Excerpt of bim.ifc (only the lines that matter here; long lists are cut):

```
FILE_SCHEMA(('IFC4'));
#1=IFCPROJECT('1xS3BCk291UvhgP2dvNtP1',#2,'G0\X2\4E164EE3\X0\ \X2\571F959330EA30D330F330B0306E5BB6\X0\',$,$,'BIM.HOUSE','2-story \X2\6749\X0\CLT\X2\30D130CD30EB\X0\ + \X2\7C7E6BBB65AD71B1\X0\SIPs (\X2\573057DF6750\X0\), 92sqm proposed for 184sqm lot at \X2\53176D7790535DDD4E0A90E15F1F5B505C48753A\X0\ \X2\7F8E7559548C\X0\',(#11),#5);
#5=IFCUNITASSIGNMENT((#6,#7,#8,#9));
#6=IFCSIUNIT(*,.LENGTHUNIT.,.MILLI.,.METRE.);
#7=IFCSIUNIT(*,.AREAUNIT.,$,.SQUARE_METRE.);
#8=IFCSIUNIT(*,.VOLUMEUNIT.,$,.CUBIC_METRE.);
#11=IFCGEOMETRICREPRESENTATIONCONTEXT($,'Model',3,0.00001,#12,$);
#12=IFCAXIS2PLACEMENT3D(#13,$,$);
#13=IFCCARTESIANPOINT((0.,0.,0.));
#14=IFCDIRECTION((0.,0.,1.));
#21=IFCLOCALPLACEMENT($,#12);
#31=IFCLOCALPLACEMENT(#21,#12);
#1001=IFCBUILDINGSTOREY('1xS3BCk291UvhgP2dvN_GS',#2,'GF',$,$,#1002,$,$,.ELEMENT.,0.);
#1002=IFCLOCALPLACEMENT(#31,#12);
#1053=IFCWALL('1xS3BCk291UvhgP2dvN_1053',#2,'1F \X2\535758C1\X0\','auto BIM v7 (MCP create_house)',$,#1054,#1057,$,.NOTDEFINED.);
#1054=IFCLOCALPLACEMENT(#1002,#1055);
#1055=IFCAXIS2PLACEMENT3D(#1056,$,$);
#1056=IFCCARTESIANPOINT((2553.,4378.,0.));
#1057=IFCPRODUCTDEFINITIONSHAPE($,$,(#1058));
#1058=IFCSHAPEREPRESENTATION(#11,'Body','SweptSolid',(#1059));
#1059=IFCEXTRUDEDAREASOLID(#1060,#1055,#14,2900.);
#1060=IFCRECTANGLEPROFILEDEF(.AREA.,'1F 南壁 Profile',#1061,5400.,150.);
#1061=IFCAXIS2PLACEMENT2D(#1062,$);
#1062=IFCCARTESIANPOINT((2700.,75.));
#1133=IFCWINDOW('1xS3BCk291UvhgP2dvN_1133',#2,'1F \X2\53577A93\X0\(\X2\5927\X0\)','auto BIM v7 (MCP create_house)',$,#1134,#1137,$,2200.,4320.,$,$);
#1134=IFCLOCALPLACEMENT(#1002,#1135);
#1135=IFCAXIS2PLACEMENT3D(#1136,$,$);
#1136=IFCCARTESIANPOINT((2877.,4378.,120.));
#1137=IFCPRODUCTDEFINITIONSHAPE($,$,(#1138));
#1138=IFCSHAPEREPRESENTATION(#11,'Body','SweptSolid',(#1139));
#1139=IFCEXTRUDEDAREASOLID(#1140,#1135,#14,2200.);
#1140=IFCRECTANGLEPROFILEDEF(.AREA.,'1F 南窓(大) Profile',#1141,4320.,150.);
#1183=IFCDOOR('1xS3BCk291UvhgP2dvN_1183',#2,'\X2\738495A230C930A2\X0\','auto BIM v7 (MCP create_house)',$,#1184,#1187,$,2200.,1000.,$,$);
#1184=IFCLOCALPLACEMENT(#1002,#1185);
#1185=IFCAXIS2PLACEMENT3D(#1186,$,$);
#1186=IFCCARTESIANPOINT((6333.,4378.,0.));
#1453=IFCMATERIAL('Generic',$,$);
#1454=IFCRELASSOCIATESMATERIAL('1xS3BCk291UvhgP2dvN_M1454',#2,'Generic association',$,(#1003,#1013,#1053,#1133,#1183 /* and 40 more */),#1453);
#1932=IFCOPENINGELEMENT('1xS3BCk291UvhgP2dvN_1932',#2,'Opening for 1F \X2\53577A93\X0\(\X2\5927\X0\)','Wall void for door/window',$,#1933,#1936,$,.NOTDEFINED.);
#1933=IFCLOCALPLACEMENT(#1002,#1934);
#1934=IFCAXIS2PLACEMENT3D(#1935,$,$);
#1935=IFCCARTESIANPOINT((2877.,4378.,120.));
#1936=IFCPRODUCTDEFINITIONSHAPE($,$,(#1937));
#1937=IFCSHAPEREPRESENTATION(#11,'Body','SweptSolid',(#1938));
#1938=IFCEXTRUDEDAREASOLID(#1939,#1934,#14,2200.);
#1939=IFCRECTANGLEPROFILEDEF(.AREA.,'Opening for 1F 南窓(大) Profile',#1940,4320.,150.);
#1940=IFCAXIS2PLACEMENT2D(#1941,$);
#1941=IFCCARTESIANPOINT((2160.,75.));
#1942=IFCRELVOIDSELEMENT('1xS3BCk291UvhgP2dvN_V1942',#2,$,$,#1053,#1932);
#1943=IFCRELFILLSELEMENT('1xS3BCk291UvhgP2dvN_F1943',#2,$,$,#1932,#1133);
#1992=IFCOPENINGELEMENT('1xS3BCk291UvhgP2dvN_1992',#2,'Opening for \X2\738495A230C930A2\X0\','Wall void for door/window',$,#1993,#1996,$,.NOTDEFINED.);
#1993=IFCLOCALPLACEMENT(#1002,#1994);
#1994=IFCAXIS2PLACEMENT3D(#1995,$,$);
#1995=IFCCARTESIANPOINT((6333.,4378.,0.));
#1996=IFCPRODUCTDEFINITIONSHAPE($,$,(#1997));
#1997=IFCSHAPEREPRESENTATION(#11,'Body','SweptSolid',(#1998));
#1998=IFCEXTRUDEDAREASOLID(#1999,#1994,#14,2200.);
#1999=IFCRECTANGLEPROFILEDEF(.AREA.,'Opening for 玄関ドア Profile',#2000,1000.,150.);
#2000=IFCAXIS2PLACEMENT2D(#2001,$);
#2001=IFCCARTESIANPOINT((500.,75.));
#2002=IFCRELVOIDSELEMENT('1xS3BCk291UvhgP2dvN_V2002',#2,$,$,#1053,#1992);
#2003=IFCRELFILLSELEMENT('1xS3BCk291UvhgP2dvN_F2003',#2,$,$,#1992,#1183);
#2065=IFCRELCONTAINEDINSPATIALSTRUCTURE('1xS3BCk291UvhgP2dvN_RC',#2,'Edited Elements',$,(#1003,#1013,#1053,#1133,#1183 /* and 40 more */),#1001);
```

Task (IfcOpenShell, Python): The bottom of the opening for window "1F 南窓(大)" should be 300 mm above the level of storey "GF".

```python
import numpy as np
import ifcopenshell
import ifcopenshell.api.geometry
import ifcopenshell.geom
import ifcopenshell.util.element
import ifcopenshell.util.placement
import ifcopenshell.util.shape
import ifcopenshell.util.unit

model = ifcopenshell.open("bim.ifc")
unit_scale = ifcopenshell.util.unit.calculate_unit_scale(model)

window = model.by_guid("1xS3BCk291UvhgP2dvN_1133")
opening = window.FillsVoids[0].RelatingOpeningElement
storey = ifcopenshell.util.element.get_container(window, ifc_class="IfcBuildingStorey")
level = ifcopenshell.util.placement.get_local_placement(storey.ObjectPlacement)[2, 3]

# The opening's origin need not be at the sill, so measure its lowest point.
shape = ifcopenshell.geom.create_shape(ifcopenshell.geom.settings(), opening)
bottom = ifcopenshell.util.shape.get_shape_bottom_elevation(shape, shape.geometry) / unit_scale
dz = level + 0.3 / unit_scale - bottom

shift = np.array([0.0, 0.0, dz])
# The window is not placed relative to its opening, so move both.
for product in (opening, window):
    matrix = ifcopenshell.util.placement.get_local_placement(product.ObjectPlacement)
    matrix[:3, 3] += shift
    ifcopenshell.api.geometry.edit_object_placement(model, product=product, matrix=matrix, is_si=False)

print(f"moved by {dz * unit_scale:+.3f} m")

model.write("bim_updated.ifc")
```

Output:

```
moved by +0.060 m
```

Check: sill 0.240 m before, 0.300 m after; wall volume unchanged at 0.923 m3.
